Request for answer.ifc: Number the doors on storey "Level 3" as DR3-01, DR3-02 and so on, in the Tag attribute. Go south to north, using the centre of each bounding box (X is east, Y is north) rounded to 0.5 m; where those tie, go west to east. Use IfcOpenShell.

First a look at what the model holds.

```python
import ifcopenshell
import ifcopenshell.util.element
import ifcopenshell.util.placement

model = ifcopenshell.open("answer.ifc")
print(model.schema)
storey = next(s for s in model.by_type("IfcBuildingStorey") if s.Name == "Level 3")
doors = [e for e in ifcopenshell.util.element.get_decomposition(storey) if e.is_a("IfcDoor")]
for e in sorted(doors, key=lambda e: e.id()):
    origin = ifcopenshell.util.placement.get_local_placement(e.ObjectPlacement)[:3, 3]
    print(e.id(), e.Tag, e.Name, origin.round(2) + 0.0, sep=" | ")
```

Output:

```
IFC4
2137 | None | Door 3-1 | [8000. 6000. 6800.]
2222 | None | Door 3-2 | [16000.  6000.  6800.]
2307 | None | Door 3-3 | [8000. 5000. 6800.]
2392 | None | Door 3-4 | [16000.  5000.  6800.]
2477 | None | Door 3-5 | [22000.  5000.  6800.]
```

```python
import ifcopenshell
import ifcopenshell.geom
import ifcopenshell.util.element
import ifcopenshell.util.shape

model = ifcopenshell.open("answer.ifc")
settings = ifcopenshell.geom.settings()
settings.set("use-world-coords", True)


def centre(element):
    shape = ifcopenshell.geom.create_shape(settings, element)
    return ifcopenshell.util.shape.get_bbox_centroid(shape.geometry)


storey = next(s for s in model.by_type("IfcBuildingStorey") if s.Name == "Level 3")
doors = [e for e in ifcopenshell.util.element.get_decomposition(storey) if e.is_a("IfcDoor")]

# Insertion points can sit at a corner or the storey origin, so sort by the geometry (in metres).
centres = {e: centre(e) for e in doors}
doors.sort(key=lambda e: (round(centres[e][1] / 0.5), centres[e][0]))

for i, e in enumerate(doors, start=1):
    number = f"DR3-{i:02d}"
    e.Tag = number
    print(e.id(), number)

model.write("answer_updated.ifc")
```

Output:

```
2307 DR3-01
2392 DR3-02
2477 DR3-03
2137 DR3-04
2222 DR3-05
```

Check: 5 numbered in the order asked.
